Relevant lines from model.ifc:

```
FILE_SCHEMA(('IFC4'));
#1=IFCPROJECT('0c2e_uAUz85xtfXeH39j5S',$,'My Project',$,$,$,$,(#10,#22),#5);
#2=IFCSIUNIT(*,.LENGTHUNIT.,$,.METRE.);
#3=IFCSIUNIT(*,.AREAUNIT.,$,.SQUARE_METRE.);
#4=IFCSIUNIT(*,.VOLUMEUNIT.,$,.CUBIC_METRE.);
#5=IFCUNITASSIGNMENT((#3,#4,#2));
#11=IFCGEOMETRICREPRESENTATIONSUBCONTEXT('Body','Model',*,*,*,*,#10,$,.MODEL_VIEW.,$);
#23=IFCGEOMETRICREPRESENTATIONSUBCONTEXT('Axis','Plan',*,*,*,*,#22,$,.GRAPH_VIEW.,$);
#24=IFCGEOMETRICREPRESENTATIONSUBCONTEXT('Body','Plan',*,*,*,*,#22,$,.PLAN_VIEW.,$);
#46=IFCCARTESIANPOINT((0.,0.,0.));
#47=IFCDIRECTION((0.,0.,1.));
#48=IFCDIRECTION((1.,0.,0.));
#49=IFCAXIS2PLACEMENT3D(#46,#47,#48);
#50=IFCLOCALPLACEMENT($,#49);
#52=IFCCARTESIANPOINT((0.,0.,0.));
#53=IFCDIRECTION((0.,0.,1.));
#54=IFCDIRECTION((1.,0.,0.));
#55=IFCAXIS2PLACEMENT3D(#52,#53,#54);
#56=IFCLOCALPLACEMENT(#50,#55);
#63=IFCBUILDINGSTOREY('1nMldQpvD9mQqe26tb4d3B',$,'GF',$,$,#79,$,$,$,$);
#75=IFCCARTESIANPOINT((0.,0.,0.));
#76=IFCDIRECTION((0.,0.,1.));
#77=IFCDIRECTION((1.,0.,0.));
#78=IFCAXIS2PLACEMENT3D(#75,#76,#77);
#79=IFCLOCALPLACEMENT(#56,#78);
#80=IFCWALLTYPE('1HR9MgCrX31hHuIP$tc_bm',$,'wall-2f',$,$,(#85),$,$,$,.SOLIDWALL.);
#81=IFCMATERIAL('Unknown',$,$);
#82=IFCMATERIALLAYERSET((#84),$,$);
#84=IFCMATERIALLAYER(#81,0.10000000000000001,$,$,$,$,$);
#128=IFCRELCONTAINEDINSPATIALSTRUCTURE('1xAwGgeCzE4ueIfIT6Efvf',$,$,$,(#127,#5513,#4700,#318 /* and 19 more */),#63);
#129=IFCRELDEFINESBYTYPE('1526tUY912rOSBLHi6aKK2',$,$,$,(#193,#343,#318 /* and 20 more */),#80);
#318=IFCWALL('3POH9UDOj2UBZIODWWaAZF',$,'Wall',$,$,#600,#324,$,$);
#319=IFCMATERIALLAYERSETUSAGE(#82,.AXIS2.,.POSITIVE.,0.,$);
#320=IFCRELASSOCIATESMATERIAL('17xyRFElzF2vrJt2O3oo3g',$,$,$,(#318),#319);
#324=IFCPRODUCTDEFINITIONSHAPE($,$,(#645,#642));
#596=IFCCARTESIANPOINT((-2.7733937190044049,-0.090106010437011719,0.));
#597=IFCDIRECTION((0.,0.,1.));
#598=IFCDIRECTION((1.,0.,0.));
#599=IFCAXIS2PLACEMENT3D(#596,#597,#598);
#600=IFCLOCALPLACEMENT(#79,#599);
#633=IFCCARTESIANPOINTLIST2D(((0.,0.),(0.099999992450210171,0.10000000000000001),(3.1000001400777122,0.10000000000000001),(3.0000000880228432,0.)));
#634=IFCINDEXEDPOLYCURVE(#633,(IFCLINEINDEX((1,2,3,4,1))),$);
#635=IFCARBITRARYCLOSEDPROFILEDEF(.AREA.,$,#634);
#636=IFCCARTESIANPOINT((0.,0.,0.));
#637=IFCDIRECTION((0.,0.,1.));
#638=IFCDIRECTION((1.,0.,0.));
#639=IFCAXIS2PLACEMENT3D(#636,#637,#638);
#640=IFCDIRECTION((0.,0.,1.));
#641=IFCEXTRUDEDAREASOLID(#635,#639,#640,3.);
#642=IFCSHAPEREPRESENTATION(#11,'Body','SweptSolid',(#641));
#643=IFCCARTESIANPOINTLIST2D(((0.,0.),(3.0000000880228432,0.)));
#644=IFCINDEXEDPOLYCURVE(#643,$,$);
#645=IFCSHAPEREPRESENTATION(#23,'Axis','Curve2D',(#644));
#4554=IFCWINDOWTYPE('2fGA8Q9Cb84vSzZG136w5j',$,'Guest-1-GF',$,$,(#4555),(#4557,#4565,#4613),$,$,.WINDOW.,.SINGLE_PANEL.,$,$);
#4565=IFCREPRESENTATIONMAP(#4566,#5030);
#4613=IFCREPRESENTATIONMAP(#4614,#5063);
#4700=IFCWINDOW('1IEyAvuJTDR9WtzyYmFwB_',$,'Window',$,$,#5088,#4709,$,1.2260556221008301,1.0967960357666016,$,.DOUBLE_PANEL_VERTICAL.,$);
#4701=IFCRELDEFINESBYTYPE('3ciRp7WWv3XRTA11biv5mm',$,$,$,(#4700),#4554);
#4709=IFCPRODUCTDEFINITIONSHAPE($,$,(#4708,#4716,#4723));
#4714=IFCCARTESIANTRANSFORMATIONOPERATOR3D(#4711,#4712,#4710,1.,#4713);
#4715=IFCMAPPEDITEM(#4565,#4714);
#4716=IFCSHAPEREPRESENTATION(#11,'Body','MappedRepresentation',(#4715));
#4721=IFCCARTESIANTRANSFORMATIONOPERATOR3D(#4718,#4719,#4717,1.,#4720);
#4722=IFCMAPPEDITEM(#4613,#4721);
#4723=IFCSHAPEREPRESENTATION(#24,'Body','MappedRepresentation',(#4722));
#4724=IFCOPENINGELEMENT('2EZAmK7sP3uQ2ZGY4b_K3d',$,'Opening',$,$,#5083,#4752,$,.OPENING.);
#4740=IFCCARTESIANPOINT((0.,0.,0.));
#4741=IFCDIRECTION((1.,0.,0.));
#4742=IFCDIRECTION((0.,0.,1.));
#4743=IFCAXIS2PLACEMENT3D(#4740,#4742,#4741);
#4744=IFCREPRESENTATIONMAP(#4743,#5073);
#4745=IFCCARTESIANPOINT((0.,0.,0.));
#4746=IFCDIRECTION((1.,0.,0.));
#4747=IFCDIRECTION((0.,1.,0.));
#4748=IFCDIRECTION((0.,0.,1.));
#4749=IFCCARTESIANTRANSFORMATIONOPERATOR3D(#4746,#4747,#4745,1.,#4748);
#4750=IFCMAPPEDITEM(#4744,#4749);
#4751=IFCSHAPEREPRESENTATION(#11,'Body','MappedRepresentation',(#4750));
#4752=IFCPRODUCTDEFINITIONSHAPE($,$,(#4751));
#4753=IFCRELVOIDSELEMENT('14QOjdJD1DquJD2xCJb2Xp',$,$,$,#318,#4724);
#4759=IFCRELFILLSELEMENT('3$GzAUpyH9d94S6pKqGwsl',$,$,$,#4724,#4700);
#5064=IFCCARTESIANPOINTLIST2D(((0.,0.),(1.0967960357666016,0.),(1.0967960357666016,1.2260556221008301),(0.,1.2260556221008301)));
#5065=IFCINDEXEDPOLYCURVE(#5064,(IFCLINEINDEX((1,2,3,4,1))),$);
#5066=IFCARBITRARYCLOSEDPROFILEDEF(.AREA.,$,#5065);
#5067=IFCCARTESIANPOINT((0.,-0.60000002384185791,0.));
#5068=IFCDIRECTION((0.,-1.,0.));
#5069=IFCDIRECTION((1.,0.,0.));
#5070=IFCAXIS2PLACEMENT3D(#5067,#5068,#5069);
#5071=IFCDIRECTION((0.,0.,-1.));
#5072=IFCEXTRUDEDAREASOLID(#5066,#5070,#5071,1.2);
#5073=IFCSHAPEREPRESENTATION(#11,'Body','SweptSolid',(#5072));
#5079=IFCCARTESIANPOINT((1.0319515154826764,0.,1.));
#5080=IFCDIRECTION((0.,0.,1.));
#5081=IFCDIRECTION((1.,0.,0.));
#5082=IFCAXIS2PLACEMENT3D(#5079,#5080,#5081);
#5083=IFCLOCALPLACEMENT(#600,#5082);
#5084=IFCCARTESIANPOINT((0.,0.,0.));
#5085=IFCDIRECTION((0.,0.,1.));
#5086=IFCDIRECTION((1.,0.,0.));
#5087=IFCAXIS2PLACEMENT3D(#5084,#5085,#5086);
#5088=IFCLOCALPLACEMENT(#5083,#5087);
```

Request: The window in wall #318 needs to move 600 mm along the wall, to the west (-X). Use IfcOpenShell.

```python
import ifcopenshell
import ifcopenshell.api.geometry
import ifcopenshell.util.placement
import ifcopenshell.util.unit

model = ifcopenshell.open("model.ifc")
unit_scale = ifcopenshell.util.unit.calculate_unit_scale(model)

window = model.by_guid("1IEyAvuJTDR9WtzyYmFwB_")
opening = window.FillsVoids[0].RelatingOpeningElement
wall = opening.VoidsElements[0].RelatingBuildingElement

wall_matrix = ifcopenshell.util.placement.get_local_placement(wall.ObjectPlacement)
shift = wall_matrix[:3, 0] * -0.6 / unit_scale
before = ifcopenshell.util.placement.get_local_placement(window.ObjectPlacement)[:3, 3].copy()

# The window is placed relative to its opening, so it follows when the opening moves.
matrix = ifcopenshell.util.placement.get_local_placement(opening.ObjectPlacement)
matrix[:3, 3] += shift
ifcopenshell.api.geometry.edit_object_placement(
    model, product=opening, matrix=matrix, is_si=False, should_transform_children=True
)

after = ifcopenshell.util.placement.get_local_placement(window.ObjectPlacement)[:3, 3]
print("window moved by", (after - before).round(3) + 0.0)

model.write("model_edited.ifc")
```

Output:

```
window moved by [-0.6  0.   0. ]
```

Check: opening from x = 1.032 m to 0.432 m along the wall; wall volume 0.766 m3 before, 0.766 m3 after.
